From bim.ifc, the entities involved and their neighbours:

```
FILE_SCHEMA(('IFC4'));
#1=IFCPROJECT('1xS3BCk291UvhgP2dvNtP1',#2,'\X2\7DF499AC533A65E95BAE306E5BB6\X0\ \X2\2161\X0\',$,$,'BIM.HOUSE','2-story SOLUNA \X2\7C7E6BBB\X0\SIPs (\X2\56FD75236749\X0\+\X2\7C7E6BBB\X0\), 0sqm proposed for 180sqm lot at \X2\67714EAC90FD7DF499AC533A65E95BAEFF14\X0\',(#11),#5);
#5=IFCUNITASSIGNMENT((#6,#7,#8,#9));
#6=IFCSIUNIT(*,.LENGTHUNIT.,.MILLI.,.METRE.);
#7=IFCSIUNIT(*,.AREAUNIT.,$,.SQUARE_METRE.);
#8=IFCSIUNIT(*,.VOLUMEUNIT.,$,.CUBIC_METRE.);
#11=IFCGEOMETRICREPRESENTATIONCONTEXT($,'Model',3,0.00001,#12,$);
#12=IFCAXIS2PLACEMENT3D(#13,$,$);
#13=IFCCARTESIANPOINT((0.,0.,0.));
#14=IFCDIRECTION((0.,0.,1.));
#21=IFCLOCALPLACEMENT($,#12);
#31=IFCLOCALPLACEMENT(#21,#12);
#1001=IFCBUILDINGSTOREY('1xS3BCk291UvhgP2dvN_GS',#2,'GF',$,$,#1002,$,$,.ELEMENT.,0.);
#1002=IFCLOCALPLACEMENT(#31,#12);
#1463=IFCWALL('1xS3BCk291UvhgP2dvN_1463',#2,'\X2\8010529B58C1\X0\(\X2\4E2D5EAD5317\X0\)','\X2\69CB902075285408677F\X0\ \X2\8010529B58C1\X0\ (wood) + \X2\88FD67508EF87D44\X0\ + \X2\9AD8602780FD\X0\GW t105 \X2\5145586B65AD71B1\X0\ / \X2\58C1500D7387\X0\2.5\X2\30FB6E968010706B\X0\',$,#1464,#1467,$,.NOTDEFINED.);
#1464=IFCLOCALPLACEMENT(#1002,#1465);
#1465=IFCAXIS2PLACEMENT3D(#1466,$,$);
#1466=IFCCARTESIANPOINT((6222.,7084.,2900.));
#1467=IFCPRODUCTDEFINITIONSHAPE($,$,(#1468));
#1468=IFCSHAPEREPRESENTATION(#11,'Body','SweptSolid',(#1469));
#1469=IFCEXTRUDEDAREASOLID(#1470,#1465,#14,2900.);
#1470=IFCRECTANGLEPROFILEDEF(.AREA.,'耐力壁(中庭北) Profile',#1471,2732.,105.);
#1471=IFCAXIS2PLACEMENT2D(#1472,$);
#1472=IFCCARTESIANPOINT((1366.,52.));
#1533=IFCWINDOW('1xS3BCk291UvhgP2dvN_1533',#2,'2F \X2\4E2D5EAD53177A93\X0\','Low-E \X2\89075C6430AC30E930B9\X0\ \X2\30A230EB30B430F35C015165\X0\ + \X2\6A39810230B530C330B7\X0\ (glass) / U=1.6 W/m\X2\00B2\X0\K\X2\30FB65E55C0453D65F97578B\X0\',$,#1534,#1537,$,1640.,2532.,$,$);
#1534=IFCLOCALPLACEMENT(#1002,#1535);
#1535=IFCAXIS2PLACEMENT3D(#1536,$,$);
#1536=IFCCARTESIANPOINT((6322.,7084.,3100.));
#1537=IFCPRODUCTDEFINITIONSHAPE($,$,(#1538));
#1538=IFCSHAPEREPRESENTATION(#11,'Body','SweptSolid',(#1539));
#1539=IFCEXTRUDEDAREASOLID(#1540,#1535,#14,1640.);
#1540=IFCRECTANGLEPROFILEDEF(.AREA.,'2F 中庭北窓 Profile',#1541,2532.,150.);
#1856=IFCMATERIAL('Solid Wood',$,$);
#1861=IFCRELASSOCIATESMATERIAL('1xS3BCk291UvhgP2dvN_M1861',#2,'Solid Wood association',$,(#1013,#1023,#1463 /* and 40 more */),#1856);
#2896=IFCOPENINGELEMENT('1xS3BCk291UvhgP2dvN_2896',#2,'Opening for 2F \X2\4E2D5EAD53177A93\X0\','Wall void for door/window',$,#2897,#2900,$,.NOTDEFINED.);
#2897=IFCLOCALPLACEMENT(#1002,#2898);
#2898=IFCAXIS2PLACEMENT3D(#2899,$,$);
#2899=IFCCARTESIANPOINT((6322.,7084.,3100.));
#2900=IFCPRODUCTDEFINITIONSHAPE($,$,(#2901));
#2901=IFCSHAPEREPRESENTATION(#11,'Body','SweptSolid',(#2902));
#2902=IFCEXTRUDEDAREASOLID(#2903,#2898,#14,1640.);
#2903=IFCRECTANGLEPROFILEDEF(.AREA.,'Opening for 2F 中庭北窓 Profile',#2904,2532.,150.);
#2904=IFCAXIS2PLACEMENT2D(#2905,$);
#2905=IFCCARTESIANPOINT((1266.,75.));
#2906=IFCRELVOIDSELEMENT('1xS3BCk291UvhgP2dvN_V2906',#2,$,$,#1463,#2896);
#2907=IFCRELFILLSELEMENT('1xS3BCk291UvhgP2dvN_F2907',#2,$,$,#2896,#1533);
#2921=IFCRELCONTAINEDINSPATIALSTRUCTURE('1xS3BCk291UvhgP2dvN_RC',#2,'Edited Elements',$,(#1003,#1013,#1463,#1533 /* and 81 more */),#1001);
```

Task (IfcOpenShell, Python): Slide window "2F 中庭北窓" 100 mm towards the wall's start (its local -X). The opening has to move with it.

```python
import ifcopenshell
import ifcopenshell.api.geometry
import ifcopenshell.util.placement
import ifcopenshell.util.unit

model = ifcopenshell.open("bim.ifc")
unit_scale = ifcopenshell.util.unit.calculate_unit_scale(model)

window = model.by_id(1533)
opening = window.FillsVoids[0].RelatingOpeningElement
wall = opening.VoidsElements[0].RelatingBuildingElement

wall_matrix = ifcopenshell.util.placement.get_local_placement(wall.ObjectPlacement)
shift = wall_matrix[:3, 0] * -0.1 / unit_scale
before = ifcopenshell.util.placement.get_local_placement(window.ObjectPlacement)[:3, 3].copy()

# The window is not placed relative to its opening, so move both.
for product in (opening, window):
    matrix = ifcopenshell.util.placement.get_local_placement(product.ObjectPlacement)
    matrix[:3, 3] += shift
    ifcopenshell.api.geometry.edit_object_placement(model, product=product, matrix=matrix, is_si=False)

after = ifcopenshell.util.placement.get_local_placement(window.ObjectPlacement)[:3, 3]
print("window moved by", (after - before).round(3) + 0.0)

model.write("bim-out.ifc")
```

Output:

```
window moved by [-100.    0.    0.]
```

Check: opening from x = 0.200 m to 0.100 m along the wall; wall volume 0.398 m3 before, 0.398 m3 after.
